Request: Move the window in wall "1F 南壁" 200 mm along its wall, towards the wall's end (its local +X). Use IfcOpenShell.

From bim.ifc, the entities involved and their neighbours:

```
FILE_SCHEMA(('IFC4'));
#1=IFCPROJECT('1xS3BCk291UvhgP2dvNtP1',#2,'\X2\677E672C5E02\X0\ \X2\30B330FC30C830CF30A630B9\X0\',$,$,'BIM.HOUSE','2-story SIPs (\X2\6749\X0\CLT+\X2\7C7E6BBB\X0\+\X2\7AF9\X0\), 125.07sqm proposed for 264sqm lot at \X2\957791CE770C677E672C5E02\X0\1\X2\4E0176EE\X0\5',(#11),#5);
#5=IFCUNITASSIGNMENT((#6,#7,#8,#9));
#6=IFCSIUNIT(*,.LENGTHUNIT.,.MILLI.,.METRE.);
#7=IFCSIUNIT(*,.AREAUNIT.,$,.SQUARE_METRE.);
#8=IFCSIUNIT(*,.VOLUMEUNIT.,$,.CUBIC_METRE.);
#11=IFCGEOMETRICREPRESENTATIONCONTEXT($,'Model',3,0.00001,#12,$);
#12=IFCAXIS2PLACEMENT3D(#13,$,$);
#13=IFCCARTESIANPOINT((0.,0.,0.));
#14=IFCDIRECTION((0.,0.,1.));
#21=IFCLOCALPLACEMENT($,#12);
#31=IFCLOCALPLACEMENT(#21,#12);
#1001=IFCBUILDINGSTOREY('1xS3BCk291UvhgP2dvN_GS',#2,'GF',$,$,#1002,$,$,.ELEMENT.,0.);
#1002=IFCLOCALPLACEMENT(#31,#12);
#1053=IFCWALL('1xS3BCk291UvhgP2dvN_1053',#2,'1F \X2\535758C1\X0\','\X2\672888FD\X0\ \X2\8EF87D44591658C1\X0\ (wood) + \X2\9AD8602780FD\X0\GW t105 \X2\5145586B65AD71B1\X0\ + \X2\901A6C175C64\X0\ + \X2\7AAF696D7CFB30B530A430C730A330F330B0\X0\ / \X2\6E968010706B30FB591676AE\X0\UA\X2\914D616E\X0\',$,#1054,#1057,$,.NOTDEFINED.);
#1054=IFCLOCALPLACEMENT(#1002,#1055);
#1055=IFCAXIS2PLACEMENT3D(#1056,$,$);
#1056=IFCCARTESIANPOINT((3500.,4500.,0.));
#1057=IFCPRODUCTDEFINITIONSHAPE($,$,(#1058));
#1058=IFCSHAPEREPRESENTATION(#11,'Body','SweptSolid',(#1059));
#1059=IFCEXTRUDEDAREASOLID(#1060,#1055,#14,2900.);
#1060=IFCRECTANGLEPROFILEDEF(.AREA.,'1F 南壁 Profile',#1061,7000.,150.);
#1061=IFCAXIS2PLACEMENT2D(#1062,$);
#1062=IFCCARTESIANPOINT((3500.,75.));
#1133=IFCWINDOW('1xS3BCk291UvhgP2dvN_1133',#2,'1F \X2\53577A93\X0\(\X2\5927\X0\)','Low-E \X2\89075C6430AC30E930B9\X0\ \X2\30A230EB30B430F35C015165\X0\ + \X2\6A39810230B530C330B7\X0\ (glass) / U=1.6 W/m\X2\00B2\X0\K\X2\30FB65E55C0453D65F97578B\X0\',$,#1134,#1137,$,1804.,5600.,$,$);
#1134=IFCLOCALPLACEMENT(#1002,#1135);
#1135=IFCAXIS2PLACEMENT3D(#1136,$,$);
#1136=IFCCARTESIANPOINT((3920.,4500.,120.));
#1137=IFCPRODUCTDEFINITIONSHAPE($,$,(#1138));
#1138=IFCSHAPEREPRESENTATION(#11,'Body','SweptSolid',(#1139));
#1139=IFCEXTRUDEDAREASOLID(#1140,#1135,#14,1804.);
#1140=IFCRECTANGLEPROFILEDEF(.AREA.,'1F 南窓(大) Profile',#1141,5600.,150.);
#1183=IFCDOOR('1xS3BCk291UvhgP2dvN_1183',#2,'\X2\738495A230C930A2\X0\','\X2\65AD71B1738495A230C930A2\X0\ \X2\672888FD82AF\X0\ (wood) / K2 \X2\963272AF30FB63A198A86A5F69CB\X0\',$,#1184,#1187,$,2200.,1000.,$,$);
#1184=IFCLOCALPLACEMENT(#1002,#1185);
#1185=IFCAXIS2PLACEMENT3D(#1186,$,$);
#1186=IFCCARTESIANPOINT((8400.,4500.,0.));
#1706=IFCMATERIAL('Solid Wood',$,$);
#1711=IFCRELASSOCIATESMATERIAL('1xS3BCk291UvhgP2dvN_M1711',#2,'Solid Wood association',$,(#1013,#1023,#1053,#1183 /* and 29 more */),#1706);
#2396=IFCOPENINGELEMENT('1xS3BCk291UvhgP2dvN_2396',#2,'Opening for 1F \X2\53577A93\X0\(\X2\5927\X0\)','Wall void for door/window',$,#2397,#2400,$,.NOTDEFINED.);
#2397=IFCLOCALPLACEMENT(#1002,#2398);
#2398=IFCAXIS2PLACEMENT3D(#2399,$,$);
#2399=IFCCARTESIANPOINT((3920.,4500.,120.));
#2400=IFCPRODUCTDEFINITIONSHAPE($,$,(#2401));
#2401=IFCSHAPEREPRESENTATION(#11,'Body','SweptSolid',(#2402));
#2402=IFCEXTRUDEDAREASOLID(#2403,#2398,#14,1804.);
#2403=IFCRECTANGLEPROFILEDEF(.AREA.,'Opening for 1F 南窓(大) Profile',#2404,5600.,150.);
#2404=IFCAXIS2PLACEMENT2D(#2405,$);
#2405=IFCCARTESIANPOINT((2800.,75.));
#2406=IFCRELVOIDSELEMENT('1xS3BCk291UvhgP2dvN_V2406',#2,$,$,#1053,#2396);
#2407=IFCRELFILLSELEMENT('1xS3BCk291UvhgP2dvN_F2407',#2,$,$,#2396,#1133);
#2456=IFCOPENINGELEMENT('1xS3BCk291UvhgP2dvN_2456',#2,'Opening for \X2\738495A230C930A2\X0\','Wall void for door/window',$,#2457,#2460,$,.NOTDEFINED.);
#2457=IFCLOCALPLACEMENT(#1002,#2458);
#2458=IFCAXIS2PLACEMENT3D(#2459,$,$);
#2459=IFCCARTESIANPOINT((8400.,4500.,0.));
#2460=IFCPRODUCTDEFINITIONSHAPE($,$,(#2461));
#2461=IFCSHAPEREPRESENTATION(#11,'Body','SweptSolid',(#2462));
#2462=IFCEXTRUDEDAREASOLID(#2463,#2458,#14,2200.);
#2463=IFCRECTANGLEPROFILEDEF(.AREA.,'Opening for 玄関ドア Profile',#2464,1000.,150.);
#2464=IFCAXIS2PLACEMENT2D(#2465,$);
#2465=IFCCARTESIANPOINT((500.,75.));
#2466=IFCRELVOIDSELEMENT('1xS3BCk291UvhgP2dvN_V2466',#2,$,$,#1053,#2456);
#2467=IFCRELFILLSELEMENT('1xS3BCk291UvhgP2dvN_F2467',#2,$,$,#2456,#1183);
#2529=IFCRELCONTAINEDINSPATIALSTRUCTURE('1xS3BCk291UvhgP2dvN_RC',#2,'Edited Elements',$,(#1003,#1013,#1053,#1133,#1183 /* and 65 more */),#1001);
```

```python
import ifcopenshell
import ifcopenshell.api.geometry
import ifcopenshell.util.placement

model = ifcopenshell.open("bim.ifc")

window = model.by_guid("1xS3BCk291UvhgP2dvN_1133")
opening = window.FillsVoids[0].RelatingOpeningElement
wall = opening.VoidsElements[0].RelatingBuildingElement

wall_matrix = ifcopenshell.util.placement.get_local_placement(wall.ObjectPlacement)
shift = wall_matrix[:3, 0] * 200.0
before = ifcopenshell.util.placement.get_local_placement(window.ObjectPlacement)[:3, 3].copy()

# The window is not placed relative to its opening, so move both.
for product in (opening, window):
    matrix = ifcopenshell.util.placement.get_local_placement(product.ObjectPlacement)
    matrix[:3, 3] += shift
    ifcopenshell.api.geometry.edit_object_placement(model, product=product, matrix=matrix, is_si=False)

after = ifcopenshell.util.placement.get_local_placement(window.ObjectPlacement)[:3, 3]
print("window moved by", (after - before).round(3) + 0.0)

model.write("bim_rev.ifc")
```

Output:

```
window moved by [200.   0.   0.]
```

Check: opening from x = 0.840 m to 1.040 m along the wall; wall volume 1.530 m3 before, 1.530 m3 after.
